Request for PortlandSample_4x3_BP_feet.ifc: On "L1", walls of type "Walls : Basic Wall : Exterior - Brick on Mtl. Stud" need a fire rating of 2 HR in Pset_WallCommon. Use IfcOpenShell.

First a look at what the model holds.

```python
import ifcopenshell
import ifcopenshell.util.element

model = ifcopenshell.open("PortlandSample_4x3_BP_feet.ifc")
print(model.schema)
storey = next(s for s in model.by_type("IfcBuildingStorey") if s.Name == "L1")
walls = [e for e in ifcopenshell.util.element.get_decomposition(storey) if e.is_a("IfcWall")]
seen = {}
for e in walls:
    element_type = ifcopenshell.util.element.get_type(e)
    key = (element_type.Name if element_type != e and element_type else None, ifcopenshell.util.element.get_pset(e, "Pset_WallCommon", "FireRating"))
    seen[key] = seen.get(key, 0) + 1
for (name, value), count in sorted(seen.items(), key=str):
    print(count, "x", name, "|", value)
```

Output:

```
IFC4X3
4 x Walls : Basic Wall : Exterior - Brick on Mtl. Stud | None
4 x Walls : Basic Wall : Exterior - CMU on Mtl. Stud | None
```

```python
import ifcopenshell
import ifcopenshell.api.pset
import ifcopenshell.util.element

model = ifcopenshell.open("PortlandSample_4x3_BP_feet.ifc")

storey = next(s for s in model.by_type("IfcBuildingStorey") if s.Name == "L1")
walls = [e for e in ifcopenshell.util.element.get_decomposition(storey) if e.is_a("IfcWall")]

count = 0
for e in walls:
    element_type = ifcopenshell.util.element.get_type(e)
    if element_type in (None, e) or element_type.Name != "Walls : Basic Wall : Exterior - Brick on Mtl. Stud":
        continue
    # add_pset returns the element's existing set when there is one.
    pset = ifcopenshell.api.pset.add_pset(model, product=e, name="Pset_WallCommon")
    ifcopenshell.api.pset.edit_pset(model, pset=pset, properties={"FireRating": "2 HR"})
    count += 1

print(count, "walls updated")

model.write("PortlandSample_4x3_BP_feet_updated.ifc")
```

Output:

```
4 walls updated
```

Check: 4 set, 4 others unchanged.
